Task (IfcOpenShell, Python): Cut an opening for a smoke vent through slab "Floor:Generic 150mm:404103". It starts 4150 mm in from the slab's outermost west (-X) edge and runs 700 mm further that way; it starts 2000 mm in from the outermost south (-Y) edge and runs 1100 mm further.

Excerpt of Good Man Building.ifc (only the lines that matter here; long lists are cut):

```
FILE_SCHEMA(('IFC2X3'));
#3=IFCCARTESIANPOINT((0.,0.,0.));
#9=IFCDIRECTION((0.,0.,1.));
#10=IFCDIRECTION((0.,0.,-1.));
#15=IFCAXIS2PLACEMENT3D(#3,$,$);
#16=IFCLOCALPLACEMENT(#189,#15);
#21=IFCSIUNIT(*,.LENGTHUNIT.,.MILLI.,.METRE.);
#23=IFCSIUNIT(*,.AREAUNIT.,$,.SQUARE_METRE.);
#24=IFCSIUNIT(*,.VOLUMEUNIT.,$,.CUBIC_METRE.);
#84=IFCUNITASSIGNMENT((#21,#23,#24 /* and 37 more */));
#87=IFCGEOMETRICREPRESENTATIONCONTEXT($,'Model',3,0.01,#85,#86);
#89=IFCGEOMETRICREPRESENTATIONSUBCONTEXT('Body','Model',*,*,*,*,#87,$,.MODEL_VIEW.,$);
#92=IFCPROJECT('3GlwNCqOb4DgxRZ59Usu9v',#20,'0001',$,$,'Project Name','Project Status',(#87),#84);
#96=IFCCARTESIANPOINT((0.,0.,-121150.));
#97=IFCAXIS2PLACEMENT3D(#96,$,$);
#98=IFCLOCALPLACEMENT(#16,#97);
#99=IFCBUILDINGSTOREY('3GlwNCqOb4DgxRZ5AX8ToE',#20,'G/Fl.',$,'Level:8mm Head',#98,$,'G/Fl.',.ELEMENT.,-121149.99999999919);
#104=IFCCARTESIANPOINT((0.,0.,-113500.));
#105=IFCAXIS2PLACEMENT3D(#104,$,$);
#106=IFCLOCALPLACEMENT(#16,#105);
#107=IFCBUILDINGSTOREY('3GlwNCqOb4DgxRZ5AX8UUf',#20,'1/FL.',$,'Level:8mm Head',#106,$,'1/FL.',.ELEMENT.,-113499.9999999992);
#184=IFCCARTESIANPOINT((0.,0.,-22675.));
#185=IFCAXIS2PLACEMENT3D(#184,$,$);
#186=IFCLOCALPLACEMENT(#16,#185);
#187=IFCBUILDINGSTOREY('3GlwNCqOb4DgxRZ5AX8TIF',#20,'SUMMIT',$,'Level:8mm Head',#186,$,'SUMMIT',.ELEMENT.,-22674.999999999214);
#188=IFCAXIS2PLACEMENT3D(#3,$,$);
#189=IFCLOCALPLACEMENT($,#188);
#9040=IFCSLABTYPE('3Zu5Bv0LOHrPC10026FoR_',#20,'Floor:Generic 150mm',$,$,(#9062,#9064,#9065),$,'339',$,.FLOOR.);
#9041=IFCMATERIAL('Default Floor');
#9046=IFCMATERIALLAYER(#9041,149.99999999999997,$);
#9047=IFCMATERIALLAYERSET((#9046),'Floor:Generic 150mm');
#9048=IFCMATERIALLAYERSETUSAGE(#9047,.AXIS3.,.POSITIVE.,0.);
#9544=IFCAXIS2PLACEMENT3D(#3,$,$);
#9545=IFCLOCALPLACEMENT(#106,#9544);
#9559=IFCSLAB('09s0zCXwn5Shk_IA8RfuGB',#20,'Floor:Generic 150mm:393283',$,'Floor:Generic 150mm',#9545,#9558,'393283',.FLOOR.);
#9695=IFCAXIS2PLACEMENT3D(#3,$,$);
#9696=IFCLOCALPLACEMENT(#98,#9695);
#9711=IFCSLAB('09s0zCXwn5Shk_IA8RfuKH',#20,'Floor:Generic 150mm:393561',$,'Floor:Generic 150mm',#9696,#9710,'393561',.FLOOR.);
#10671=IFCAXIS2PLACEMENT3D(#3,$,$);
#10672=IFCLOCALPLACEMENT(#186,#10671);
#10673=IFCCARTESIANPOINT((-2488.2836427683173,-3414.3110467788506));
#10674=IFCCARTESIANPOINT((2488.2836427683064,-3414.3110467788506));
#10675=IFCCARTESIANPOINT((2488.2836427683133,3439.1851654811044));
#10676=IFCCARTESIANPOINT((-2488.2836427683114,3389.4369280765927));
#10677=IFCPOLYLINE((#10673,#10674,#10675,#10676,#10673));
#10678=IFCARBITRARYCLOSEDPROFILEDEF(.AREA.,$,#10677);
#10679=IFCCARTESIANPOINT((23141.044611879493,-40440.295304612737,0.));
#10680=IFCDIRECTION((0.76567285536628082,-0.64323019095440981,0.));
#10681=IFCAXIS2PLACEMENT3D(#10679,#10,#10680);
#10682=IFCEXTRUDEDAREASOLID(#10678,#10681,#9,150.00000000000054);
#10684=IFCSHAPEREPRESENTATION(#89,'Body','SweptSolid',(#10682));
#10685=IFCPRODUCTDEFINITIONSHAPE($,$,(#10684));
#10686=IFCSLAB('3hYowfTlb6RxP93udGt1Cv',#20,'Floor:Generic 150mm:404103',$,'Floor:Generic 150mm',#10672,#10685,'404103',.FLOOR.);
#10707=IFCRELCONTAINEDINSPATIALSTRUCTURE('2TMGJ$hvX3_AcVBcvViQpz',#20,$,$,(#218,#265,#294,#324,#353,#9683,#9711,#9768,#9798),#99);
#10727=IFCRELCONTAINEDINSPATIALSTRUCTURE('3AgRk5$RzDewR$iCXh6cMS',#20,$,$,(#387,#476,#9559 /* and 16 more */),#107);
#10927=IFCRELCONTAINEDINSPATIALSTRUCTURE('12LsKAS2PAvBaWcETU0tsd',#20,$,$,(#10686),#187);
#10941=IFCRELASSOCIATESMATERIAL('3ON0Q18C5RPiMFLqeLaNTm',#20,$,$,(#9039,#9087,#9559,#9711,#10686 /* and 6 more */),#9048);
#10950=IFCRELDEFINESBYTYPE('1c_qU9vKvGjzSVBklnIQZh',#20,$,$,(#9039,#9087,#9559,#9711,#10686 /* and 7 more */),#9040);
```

```python
import numpy as np
import ifcopenshell
import ifcopenshell.api.feature
import ifcopenshell.api.geometry
import ifcopenshell.api.root
import ifcopenshell.geom
import ifcopenshell.util.placement
import ifcopenshell.util.representation
import ifcopenshell.util.shape
import ifcopenshell.util.unit

model = ifcopenshell.open("Good Man Building.ifc")
unit_scale = ifcopenshell.util.unit.calculate_unit_scale(model)
settings = ifcopenshell.geom.settings()


def volume(element):
    """Net volume in cubic metres, openings subtracted."""
    shape = ifcopenshell.geom.create_shape(settings, element)
    return ifcopenshell.util.shape.get_volume(shape.geometry)


slab = model.by_guid("3hYowfTlb6RxP93udGt1Cv")
before = volume(slab)

# Extent in the slab's own axes, in metres. The edges named are its -X and -Y sides.
slab_shape = ifcopenshell.geom.create_shape(settings, slab)
vertices = ifcopenshell.util.shape.get_vertices(slab_shape.geometry)
x_min, y_min, bottom = vertices.min(axis=0)
top = vertices[:, 2].max()

opening = ifcopenshell.api.root.create_entity(model, ifc_class="IfcOpeningElement", name="Smoke vent opening")
context = ifcopenshell.util.representation.get_context(model, "Model", "Body", "MODEL_VIEW")
width, depth = 0.7, 1.1
outline = [(0.0, 0.0), (width, 0.0), (width, depth), (0.0, depth), (0.0, 0.0)]
# Overshoot both faces by 50 mm so the cut is clean.
shape = ifcopenshell.api.geometry.add_slab_representation(
    model, context=context, depth=top - bottom + 0.1, polyline=outline
)
ifcopenshell.api.geometry.assign_representation(model, product=opening, representation=shape)

matrix = ifcopenshell.util.placement.get_local_placement(slab.ObjectPlacement)
matrix[:, 3] = matrix @ np.append(np.array([x_min + 4.15, y_min + 2, bottom - 0.05]) / unit_scale, 1.0)
ifcopenshell.api.geometry.edit_object_placement(model, product=opening, matrix=matrix, is_si=False)
ifcopenshell.api.feature.add_feature(model, feature=opening, element=slab)

after = volume(slab)

print(f"slab volume {before:.3f} -> {after:.3f} m3")

model.write("Good Man Building_edited.ifc")
```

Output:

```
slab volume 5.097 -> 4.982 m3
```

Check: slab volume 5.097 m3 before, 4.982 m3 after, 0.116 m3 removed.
